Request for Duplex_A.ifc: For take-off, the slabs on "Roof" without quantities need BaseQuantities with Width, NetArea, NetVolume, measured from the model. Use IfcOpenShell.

First a look at what the model holds.

```python
import ifcopenshell
import ifcopenshell.util.element
import ifcopenshell.util.unit

model = ifcopenshell.open("Duplex_A.ifc")
print(model.schema)
for unit_type in ("LENGTHUNIT", "AREAUNIT", "VOLUMEUNIT"):
    print(unit_type, ifcopenshell.util.unit.calculate_unit_scale(model, unit_type))
storey = next(s for s in model.by_type("IfcBuildingStorey") if s.Name == "Roof")
slabs = [e for e in ifcopenshell.util.element.get_decomposition(storey) if e.is_a("IfcSlab")]
for e in sorted(slabs, key=lambda e: e.id()):
    print(e.id(), e.is_a(), e.Name, list(ifcopenshell.util.element.get_psets(e, qtos_only=True)), sep=" | ")
```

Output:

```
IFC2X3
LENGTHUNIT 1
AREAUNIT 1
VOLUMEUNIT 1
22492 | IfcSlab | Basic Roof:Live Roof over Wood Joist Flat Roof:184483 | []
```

```python
import ifcopenshell
import ifcopenshell.api.pset
import ifcopenshell.geom
import ifcopenshell.util.element
import ifcopenshell.util.shape
import ifcopenshell.util.unit

model = ifcopenshell.open("Duplex_A.ifc")
unit_scale = ifcopenshell.util.unit.calculate_unit_scale(model)
area_scale = ifcopenshell.util.unit.calculate_unit_scale(model, "AREAUNIT")
volume_scale = ifcopenshell.util.unit.calculate_unit_scale(model, "VOLUMEUNIT")
settings = ifcopenshell.geom.settings()

storey = next(s for s in model.by_type("IfcBuildingStorey") if s.Name == "Roof")
slabs = [e for e in ifcopenshell.util.element.get_decomposition(storey) if e.is_a("IfcSlab")]

for e in sorted(slabs, key=lambda e: e.id()):
    if ifcopenshell.util.element.get_psets(e, qtos_only=True, should_inherit=False):
        continue
    # Geometry comes back in metres, in the element's own axes.
    shape = ifcopenshell.geom.create_shape(settings, e)
    values = {
        "Width": ifcopenshell.util.shape.get_z(shape.geometry) / unit_scale,
        "NetArea": ifcopenshell.util.shape.get_footprint_area(shape.geometry) / area_scale,
        "NetVolume": ifcopenshell.util.shape.get_volume(shape.geometry) / volume_scale,
    }
    qto = ifcopenshell.api.pset.add_qto(model, product=e, name="BaseQuantities")
    ifcopenshell.api.pset.edit_qto(model, qto=qto, properties=values)
    print(e.id(), {k: round(v, 3) for k, v in values.items()})

model.write("Duplex_A_v2.ifc")
```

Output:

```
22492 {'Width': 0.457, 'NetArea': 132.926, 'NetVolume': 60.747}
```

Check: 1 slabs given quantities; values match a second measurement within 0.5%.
